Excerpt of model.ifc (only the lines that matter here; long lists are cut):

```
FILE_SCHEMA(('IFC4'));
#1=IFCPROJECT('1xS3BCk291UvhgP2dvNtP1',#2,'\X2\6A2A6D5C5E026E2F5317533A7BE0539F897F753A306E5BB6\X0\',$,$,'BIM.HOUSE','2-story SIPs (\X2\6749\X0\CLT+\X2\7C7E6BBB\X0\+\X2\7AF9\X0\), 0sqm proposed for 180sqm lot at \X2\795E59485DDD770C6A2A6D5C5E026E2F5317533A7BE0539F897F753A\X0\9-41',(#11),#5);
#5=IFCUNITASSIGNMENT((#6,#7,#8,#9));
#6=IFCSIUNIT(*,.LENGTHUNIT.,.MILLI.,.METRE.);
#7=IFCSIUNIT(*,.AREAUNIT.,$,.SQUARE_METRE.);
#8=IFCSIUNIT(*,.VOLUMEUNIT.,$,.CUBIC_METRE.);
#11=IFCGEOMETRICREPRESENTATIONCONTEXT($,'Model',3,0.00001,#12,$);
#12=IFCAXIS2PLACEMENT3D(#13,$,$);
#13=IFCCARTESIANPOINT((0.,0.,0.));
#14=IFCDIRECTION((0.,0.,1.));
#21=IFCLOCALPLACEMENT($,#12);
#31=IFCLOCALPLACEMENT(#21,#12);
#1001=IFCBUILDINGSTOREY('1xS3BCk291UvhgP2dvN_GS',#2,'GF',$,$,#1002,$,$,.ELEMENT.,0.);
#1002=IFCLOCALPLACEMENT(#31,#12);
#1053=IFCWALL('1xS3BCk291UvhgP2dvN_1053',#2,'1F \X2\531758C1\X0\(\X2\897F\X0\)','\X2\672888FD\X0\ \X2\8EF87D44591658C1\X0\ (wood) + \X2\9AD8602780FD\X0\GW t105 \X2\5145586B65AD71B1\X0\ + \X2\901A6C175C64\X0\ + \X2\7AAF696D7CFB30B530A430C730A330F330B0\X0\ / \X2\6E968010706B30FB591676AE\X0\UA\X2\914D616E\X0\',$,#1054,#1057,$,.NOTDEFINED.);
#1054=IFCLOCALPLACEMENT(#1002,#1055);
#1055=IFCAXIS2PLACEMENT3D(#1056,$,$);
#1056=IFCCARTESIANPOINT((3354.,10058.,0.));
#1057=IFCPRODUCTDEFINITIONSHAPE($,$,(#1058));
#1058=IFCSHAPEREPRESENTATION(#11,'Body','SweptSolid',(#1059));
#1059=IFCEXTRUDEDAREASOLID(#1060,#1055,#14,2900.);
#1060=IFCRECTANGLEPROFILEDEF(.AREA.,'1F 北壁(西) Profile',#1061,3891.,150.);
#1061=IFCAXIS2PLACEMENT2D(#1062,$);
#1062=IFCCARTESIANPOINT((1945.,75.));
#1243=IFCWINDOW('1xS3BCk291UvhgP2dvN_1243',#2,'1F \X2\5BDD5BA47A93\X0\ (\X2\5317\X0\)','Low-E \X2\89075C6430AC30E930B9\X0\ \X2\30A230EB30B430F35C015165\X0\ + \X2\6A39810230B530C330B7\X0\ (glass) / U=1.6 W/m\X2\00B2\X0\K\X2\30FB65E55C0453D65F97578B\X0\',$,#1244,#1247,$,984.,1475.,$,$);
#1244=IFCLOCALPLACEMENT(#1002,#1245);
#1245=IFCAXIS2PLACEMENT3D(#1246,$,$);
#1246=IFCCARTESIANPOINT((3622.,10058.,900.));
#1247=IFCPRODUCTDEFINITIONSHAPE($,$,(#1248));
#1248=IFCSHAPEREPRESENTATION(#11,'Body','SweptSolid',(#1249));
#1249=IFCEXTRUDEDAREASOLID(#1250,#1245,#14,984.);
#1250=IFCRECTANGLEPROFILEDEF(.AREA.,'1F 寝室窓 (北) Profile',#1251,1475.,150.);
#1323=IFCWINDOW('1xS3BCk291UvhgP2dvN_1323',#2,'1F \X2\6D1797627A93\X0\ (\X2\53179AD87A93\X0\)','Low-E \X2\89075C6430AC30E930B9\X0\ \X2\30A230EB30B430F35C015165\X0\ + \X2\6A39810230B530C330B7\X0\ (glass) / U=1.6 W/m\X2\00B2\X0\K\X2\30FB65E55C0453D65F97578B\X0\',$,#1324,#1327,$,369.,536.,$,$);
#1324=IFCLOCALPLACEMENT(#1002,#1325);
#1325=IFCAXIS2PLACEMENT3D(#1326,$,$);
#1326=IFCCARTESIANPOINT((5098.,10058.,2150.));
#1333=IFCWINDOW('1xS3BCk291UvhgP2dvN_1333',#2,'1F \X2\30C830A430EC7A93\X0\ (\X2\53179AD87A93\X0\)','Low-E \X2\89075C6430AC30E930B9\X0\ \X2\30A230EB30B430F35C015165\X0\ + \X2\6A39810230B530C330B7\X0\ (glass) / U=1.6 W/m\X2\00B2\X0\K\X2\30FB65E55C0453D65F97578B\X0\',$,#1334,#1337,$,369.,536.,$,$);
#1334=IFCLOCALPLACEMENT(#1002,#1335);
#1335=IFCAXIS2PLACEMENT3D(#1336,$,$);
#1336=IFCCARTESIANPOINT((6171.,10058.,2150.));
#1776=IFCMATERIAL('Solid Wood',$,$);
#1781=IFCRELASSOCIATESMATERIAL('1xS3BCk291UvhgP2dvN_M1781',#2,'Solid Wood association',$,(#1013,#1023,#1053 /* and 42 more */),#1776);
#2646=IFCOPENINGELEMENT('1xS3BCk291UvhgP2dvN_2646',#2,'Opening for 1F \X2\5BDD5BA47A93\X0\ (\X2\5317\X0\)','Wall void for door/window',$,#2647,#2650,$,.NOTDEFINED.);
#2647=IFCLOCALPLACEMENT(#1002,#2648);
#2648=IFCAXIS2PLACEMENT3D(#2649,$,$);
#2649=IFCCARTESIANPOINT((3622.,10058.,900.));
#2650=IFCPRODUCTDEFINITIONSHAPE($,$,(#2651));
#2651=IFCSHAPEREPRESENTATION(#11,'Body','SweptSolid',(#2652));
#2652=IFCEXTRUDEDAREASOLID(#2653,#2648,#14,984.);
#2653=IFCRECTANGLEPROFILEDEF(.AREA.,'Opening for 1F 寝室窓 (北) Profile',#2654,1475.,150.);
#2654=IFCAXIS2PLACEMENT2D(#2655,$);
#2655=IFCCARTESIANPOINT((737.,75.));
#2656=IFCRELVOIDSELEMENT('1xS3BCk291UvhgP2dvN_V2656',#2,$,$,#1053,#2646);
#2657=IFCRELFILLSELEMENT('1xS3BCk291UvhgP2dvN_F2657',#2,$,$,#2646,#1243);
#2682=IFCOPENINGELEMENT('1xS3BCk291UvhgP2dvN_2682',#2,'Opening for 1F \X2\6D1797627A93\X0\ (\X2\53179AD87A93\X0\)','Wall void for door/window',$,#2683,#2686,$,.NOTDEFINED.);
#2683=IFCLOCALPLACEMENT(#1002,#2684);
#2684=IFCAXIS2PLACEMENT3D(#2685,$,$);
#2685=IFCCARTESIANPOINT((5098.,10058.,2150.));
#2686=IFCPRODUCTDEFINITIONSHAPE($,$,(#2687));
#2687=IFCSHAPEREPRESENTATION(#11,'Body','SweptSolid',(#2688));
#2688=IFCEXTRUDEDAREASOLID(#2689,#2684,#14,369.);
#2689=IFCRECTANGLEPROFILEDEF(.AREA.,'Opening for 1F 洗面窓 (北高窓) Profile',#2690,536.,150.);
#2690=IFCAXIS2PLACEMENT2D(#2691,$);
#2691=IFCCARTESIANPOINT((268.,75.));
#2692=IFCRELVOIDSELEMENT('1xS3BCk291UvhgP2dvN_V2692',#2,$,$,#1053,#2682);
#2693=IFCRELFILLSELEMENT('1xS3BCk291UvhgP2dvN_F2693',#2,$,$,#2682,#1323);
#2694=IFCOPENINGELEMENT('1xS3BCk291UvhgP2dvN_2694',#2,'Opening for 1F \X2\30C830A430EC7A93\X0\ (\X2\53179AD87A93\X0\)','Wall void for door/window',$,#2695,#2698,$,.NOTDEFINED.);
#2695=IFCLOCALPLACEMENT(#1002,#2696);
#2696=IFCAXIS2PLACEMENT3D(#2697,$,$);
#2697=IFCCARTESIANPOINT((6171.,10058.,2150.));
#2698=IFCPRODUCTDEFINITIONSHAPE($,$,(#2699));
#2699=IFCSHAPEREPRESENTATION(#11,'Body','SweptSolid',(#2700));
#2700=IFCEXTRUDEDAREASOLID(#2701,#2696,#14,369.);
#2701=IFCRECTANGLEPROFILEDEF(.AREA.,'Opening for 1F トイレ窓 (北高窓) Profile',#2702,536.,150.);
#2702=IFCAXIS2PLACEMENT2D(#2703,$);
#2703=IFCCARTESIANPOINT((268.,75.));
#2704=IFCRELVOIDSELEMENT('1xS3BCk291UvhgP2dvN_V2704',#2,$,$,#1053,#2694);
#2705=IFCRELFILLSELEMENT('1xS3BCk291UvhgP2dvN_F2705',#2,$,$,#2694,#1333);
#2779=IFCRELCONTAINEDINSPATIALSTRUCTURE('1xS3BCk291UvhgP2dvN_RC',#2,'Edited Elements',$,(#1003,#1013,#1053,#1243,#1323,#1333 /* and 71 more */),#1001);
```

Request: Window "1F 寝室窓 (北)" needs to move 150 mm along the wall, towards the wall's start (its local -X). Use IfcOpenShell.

```python
import ifcopenshell
import ifcopenshell.api.geometry
import ifcopenshell.util.placement
import ifcopenshell.util.unit

model = ifcopenshell.open("model.ifc")
unit_scale = ifcopenshell.util.unit.calculate_unit_scale(model)

window = model.by_id(1243)
opening = window.FillsVoids[0].RelatingOpeningElement
wall = opening.VoidsElements[0].RelatingBuildingElement

wall_matrix = ifcopenshell.util.placement.get_local_placement(wall.ObjectPlacement)
shift = wall_matrix[:3, 0] * -0.15 / unit_scale
before = ifcopenshell.util.placement.get_local_placement(window.ObjectPlacement)[:3, 3].copy()

# The window is not placed relative to its opening, so move both.
for product in (opening, window):
    matrix = ifcopenshell.util.placement.get_local_placement(product.ObjectPlacement)
    matrix[:3, 3] += shift
    ifcopenshell.api.geometry.edit_object_placement(model, product=product, matrix=matrix, is_si=False)

after = ifcopenshell.util.placement.get_local_placement(window.ObjectPlacement)[:3, 3]
print("window moved by", (after - before).round(3) + 0.0)

model.write("model-out.ifc")
```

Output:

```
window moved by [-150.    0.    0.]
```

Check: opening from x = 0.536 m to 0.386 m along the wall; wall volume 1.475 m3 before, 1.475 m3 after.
